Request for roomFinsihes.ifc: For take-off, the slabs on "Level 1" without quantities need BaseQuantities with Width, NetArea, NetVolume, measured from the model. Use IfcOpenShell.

First a look at what the model holds.

```python
import ifcopenshell
import ifcopenshell.util.element
import ifcopenshell.util.unit

model = ifcopenshell.open("roomFinsihes.ifc")
print(model.schema)
for unit_type in ("LENGTHUNIT", "AREAUNIT", "VOLUMEUNIT"):
    print(unit_type, ifcopenshell.util.unit.calculate_unit_scale(model, unit_type))
storey = next(s for s in model.by_type("IfcBuildingStorey") if s.Name == "Level 1")
slabs = [e for e in ifcopenshell.util.element.get_decomposition(storey) if e.is_a("IfcSlab")]
for e in sorted(slabs, key=lambda e: e.id()):
    print(e.id(), e.is_a(), e.Name, list(ifcopenshell.util.element.get_psets(e, qtos_only=True)), sep=" | ")
```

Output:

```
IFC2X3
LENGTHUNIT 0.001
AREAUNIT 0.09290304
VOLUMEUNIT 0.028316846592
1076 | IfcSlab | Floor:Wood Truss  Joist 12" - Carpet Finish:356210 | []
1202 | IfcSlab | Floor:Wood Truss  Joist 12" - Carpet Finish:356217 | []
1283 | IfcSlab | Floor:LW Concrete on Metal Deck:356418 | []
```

```python
import ifcopenshell
import ifcopenshell.api.pset
import ifcopenshell.geom
import ifcopenshell.util.element
import ifcopenshell.util.shape
import ifcopenshell.util.unit

model = ifcopenshell.open("roomFinsihes.ifc")
unit_scale = ifcopenshell.util.unit.calculate_unit_scale(model)
area_scale = ifcopenshell.util.unit.calculate_unit_scale(model, "AREAUNIT")
volume_scale = ifcopenshell.util.unit.calculate_unit_scale(model, "VOLUMEUNIT")
settings = ifcopenshell.geom.settings()

storey = next(s for s in model.by_type("IfcBuildingStorey") if s.Name == "Level 1")
slabs = [e for e in ifcopenshell.util.element.get_decomposition(storey) if e.is_a("IfcSlab")]

for e in sorted(slabs, key=lambda e: e.id()):
    if ifcopenshell.util.element.get_psets(e, qtos_only=True, should_inherit=False):
        continue
    # Geometry comes back in metres, in the element's own axes.
    shape = ifcopenshell.geom.create_shape(settings, e)
    values = {
        "Width": ifcopenshell.util.shape.get_z(shape.geometry) / unit_scale,
        "NetArea": ifcopenshell.util.shape.get_footprint_area(shape.geometry) / area_scale,
        "NetVolume": ifcopenshell.util.shape.get_volume(shape.geometry) / volume_scale,
    }
    qto = ifcopenshell.api.pset.add_qto(model, product=e, name="BaseQuantities")
    ifcopenshell.api.pset.edit_qto(model, qto=qto, properties=values)
    print(e.id(), {k: round(v, 3) for k, v in values.items()})

model.write("roomFinsihes_updated.ifc")
```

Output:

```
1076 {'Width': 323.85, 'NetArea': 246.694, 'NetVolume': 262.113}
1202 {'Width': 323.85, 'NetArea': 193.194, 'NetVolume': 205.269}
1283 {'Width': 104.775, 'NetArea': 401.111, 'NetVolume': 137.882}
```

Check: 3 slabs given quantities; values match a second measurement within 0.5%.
